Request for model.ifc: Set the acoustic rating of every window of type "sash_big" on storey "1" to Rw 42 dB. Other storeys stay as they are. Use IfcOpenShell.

First a look at what the model holds.

```python
import ifcopenshell
import ifcopenshell.util.element

model = ifcopenshell.open("model.ifc")
print(model.schema)
storey = next(s for s in model.by_type("IfcBuildingStorey") if s.Name == "1")
windows = [e for e in ifcopenshell.util.element.get_decomposition(storey) if e.is_a("IfcWindow")]
seen = {}
for e in windows:
    element_type = ifcopenshell.util.element.get_type(e)
    key = (element_type.Name if element_type != e and element_type else None, ifcopenshell.util.element.get_pset(e, "Pset_WindowCommon", "AcousticRating"))
    seen[key] = seen.get(key, 0) + 1
for (name, value), count in sorted(seen.items(), key=str):
    print(count, "x", name, "|", value)
```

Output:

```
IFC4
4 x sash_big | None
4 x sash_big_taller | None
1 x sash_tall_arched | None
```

```python
import ifcopenshell
import ifcopenshell.api.pset
import ifcopenshell.util.element

model = ifcopenshell.open("model.ifc")

storey = next(s for s in model.by_type("IfcBuildingStorey") if s.Name == "1")
windows = [e for e in ifcopenshell.util.element.get_decomposition(storey) if e.is_a("IfcWindow")]

count = 0
for e in windows:
    element_type = ifcopenshell.util.element.get_type(e)
    if element_type in (None, e) or element_type.Name != "sash_big":
        continue
    # add_pset returns the element's existing set when there is one.
    pset = ifcopenshell.api.pset.add_pset(model, product=e, name="Pset_WindowCommon")
    ifcopenshell.api.pset.edit_pset(model, pset=pset, properties={"AcousticRating": "Rw 42 dB"})
    count += 1

print(count, "windows updated")

model.write("model_edited.ifc")
```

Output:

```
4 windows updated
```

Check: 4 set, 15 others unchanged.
